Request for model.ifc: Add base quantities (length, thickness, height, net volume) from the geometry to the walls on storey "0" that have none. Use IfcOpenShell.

First a look at what the model holds.

```python
import ifcopenshell
import ifcopenshell.util.element
import ifcopenshell.util.unit

model = ifcopenshell.open("model.ifc")
print(model.schema)
for unit_type in ("LENGTHUNIT", "AREAUNIT", "VOLUMEUNIT"):
    print(unit_type, ifcopenshell.util.unit.calculate_unit_scale(model, unit_type))
storey = next(s for s in model.by_type("IfcBuildingStorey") if s.Name == "0")
walls = [e for e in ifcopenshell.util.element.get_decomposition(storey) if e.is_a("IfcWall")]
for e in sorted(walls, key=lambda e: e.id()):
    print(e.id(), e.is_a(), e.Name, list(ifcopenshell.util.element.get_psets(e, qtos_only=True)), sep=" | ")
```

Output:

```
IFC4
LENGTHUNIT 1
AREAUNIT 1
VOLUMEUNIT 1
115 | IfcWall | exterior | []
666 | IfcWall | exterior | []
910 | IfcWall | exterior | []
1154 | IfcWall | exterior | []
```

```python
import ifcopenshell
import ifcopenshell.api.pset
import ifcopenshell.geom
import ifcopenshell.util.element
import ifcopenshell.util.shape
import ifcopenshell.util.unit

model = ifcopenshell.open("model.ifc")
unit_scale = ifcopenshell.util.unit.calculate_unit_scale(model)
volume_scale = ifcopenshell.util.unit.calculate_unit_scale(model, "VOLUMEUNIT")
settings = ifcopenshell.geom.settings()

storey = next(s for s in model.by_type("IfcBuildingStorey") if s.Name == "0")
walls = [e for e in ifcopenshell.util.element.get_decomposition(storey) if e.is_a("IfcWall")]

for e in sorted(walls, key=lambda e: e.id()):
    if ifcopenshell.util.element.get_psets(e, qtos_only=True, should_inherit=False):
        continue
    # Geometry comes back in metres, in the element's own axes.
    shape = ifcopenshell.geom.create_shape(settings, e)
    values = {
        "Length": ifcopenshell.util.shape.get_x(shape.geometry) / unit_scale,
        "Width": ifcopenshell.util.shape.get_y(shape.geometry) / unit_scale,
        "Height": ifcopenshell.util.shape.get_z(shape.geometry) / unit_scale,
        "NetVolume": ifcopenshell.util.shape.get_volume(shape.geometry) / volume_scale,
    }
    qto = ifcopenshell.api.pset.add_qto(model, product=e, name="Qto_WallBaseQuantities")
    ifcopenshell.api.pset.edit_qto(model, qto=qto, properties=values)
    print(e.id(), {k: round(v, 3) for k, v in values.items()})

model.write("model_edited.ifc")
```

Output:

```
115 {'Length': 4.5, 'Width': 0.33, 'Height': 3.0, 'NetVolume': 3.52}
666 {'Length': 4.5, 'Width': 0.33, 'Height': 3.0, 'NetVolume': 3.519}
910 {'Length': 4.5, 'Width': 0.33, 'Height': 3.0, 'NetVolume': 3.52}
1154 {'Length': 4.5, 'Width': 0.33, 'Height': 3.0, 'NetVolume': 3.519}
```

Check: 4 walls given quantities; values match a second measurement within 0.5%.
